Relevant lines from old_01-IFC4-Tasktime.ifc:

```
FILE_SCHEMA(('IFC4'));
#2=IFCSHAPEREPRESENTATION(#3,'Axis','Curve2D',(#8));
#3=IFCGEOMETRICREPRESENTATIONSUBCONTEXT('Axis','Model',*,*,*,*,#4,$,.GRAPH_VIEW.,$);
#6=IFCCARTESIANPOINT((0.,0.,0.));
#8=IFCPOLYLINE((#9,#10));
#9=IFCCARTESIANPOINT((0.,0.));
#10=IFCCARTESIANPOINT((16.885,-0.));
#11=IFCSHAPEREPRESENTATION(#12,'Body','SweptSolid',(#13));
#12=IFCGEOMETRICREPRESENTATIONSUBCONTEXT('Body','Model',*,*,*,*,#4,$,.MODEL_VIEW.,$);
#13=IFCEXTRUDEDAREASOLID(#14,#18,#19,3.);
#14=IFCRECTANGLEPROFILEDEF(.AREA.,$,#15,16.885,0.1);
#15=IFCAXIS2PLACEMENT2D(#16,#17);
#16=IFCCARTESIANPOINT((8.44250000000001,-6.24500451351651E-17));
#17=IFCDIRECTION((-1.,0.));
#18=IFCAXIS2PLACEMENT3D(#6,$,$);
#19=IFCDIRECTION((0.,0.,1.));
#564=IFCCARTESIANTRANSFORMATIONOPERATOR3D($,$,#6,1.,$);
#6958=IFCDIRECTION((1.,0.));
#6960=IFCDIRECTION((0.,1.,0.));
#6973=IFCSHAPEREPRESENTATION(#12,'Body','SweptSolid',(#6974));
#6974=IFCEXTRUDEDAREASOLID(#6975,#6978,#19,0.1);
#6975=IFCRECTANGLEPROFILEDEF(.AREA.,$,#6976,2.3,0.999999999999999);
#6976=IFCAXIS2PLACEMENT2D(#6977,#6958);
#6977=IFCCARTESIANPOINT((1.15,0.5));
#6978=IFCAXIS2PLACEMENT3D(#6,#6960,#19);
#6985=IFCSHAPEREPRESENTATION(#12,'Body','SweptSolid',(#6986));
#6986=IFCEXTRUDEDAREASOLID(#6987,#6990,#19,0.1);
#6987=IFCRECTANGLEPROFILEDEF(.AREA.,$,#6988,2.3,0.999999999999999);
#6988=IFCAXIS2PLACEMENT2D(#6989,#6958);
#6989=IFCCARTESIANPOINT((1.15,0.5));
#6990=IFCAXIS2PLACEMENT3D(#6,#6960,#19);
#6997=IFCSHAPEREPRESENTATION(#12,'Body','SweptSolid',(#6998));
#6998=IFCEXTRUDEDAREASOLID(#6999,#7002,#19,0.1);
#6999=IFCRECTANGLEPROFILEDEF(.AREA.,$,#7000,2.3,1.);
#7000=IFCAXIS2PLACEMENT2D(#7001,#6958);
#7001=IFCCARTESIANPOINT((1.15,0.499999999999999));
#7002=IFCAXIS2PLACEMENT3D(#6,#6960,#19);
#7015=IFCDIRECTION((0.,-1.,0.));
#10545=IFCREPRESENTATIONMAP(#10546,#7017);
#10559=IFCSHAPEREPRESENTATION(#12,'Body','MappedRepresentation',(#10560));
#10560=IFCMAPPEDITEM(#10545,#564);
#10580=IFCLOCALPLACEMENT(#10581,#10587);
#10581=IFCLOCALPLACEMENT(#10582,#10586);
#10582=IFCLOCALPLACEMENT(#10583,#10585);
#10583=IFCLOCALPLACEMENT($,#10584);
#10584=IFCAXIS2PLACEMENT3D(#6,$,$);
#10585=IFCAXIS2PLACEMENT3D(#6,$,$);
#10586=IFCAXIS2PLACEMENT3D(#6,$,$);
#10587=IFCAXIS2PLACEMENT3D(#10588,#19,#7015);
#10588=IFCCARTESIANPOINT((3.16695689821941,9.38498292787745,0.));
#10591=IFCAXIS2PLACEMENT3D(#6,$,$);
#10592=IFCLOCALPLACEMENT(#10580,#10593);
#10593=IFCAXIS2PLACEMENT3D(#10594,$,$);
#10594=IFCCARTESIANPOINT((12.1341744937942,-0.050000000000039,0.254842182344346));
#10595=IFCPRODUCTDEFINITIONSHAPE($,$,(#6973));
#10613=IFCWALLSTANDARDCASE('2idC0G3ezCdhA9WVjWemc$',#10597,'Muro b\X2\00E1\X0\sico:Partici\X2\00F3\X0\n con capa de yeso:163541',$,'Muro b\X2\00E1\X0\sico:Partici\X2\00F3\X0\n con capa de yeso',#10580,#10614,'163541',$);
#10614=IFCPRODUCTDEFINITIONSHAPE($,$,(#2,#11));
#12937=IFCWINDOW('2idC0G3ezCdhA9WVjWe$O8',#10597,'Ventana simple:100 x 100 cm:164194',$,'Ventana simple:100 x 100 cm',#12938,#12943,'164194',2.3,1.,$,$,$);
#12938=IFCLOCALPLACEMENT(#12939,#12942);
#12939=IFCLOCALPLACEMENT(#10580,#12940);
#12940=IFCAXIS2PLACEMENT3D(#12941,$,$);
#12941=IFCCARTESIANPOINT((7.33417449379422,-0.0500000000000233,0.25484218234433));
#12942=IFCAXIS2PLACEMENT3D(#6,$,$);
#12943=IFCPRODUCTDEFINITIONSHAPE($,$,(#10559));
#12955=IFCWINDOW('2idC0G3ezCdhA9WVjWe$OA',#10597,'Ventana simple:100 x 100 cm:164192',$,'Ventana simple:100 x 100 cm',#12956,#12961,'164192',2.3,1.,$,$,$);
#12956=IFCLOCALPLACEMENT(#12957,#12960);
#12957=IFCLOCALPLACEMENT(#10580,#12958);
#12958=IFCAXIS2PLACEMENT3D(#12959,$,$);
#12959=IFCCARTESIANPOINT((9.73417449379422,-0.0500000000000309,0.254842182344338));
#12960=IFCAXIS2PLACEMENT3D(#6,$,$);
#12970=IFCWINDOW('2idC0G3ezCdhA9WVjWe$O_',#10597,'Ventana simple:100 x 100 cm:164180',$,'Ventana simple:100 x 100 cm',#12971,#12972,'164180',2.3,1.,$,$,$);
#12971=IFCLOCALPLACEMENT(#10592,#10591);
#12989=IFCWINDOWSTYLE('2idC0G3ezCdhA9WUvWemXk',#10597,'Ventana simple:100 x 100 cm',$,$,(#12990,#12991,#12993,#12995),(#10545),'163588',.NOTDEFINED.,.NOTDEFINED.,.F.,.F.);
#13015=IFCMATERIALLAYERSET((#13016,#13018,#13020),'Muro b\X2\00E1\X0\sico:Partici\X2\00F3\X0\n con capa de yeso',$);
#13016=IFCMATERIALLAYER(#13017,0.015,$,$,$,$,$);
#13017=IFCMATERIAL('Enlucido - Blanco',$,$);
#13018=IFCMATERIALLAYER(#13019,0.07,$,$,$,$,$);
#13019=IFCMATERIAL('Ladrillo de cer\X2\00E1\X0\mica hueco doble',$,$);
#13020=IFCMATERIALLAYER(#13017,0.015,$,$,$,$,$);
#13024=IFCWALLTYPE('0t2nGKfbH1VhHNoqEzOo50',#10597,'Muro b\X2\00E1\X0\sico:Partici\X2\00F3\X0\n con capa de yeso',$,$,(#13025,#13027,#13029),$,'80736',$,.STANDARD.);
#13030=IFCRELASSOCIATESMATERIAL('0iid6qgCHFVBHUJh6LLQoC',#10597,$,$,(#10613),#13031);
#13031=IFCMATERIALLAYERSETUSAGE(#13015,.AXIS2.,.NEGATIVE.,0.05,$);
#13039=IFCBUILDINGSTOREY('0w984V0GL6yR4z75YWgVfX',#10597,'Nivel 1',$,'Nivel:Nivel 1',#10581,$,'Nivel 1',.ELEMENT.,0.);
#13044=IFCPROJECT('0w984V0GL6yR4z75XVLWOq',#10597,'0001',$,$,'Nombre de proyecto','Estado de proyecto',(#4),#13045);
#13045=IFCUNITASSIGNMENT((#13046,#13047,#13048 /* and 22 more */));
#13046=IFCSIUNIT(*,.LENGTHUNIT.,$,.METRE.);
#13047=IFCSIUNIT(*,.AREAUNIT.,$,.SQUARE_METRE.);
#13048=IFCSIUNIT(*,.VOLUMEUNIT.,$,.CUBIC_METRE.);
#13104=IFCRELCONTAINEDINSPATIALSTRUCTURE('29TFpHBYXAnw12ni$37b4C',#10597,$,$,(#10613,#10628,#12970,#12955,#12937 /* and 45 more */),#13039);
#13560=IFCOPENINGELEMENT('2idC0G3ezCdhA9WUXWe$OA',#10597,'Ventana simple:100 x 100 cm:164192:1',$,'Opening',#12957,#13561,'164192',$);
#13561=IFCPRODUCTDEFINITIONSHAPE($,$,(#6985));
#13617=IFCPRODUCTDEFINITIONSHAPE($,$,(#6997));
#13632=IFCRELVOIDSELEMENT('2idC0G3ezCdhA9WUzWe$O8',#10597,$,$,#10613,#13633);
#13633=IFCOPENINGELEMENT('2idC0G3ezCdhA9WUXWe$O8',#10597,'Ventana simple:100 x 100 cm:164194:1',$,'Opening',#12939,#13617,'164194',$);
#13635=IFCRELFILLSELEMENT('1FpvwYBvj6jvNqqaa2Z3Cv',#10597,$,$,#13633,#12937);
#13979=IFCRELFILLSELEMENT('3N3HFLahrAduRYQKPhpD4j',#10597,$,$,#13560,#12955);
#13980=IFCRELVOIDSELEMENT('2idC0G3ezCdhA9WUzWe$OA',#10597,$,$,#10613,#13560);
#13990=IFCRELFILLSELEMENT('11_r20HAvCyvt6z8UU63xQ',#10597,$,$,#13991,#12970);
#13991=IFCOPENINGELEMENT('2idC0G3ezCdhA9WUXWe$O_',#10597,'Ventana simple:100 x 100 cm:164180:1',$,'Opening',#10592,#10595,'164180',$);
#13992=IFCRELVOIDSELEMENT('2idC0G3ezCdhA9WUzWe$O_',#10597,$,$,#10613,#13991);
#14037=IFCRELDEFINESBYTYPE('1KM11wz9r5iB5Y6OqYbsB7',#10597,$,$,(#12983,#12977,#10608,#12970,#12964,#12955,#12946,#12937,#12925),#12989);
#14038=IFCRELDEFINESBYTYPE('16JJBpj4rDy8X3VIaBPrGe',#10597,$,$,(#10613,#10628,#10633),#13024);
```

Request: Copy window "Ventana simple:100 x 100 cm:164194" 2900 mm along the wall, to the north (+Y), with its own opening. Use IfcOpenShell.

```python
import ifcopenshell
import ifcopenshell.api.feature
import ifcopenshell.api.geometry
import ifcopenshell.api.root
import ifcopenshell.geom
import ifcopenshell.util.element
import ifcopenshell.util.placement
import ifcopenshell.util.shape
import ifcopenshell.util.unit

model = ifcopenshell.open("old_01-IFC4-Tasktime.ifc")
unit_scale = ifcopenshell.util.unit.calculate_unit_scale(model)
settings = ifcopenshell.geom.settings()


def volume(element):
    """Net volume in cubic metres, openings subtracted."""
    shape = ifcopenshell.geom.create_shape(settings, element)
    return ifcopenshell.util.shape.get_volume(shape.geometry)


def reuse_history(source, copy):
    """copy_class also copies each property set's owner history, people and application; keep the originals."""
    for rel in copy.IsDefinedBy:
        if rel.is_a("IfcRelDefinesByProperties") and (history := rel.RelatingPropertyDefinition.OwnerHistory):
            rel.RelatingPropertyDefinition.OwnerHistory = source.OwnerHistory
            ifcopenshell.util.element.remove_deep2(model, history)


window = model.by_guid("2idC0G3ezCdhA9WVjWe$O8")
opening = window.FillsVoids[0].RelatingOpeningElement
wall = opening.VoidsElements[0].RelatingBuildingElement
before = volume(wall)
shift = ifcopenshell.util.placement.get_local_placement(wall.ObjectPlacement)[:3, 0] * -2.9 / unit_scale

# copy_class copies the void relationship, type, container and properties, but no geometry.
new_opening = ifcopenshell.api.root.copy_class(model, product=opening)
new_opening.Representation = ifcopenshell.util.element.copy_deep(
    model, opening.Representation, exclude=["IfcGeometricRepresentationContext", "IfcRepresentationMap"]
)
new_opening.Name = "Ventana simple:100 x 100 cm"
new_opening.Tag = None
new_window = ifcopenshell.api.root.copy_class(model, product=window)
new_window.Representation = ifcopenshell.util.element.copy_deep(
    model, window.Representation, exclude=["IfcGeometricRepresentationContext", "IfcRepresentationMap"]
)
new_window.Name = "Ventana simple:100 x 100 cm"
new_window.Tag = None
reuse_history(window, new_window)
ifcopenshell.api.feature.add_filling(model, opening=new_opening, element=new_window)

for old, new in ((opening, new_opening), (window, new_window)):
    matrix = ifcopenshell.util.placement.get_local_placement(old.ObjectPlacement)
    matrix[:3, 3] += shift
    ifcopenshell.api.geometry.edit_object_placement(model, product=new, matrix=matrix, is_si=False)

after = volume(wall)

print(f"wall volume {before:.3f} -> {after:.3f} m3")

model.write("old_01-IFC4-Tasktime_rev.ifc")
```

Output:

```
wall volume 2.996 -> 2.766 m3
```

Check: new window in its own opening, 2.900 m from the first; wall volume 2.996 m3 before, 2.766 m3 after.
